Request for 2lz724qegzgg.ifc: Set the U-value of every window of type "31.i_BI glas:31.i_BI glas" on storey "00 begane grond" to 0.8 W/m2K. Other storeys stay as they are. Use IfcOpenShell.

First a look at what the model holds.

```python
import ifcopenshell
import ifcopenshell.util.element

model = ifcopenshell.open("2lz724qegzgg.ifc")
print(model.schema)
storey = next(s for s in model.by_type("IfcBuildingStorey") if s.Name == "00 begane grond")
windows = [e for e in ifcopenshell.util.element.get_decomposition(storey) if e.is_a("IfcWindow")]
seen = {}
for e in windows:
    element_type = ifcopenshell.util.element.get_type(e)
    key = (element_type.Name if element_type != e and element_type else None, ifcopenshell.util.element.get_pset(e, "Pset_WindowCommon", "ThermalTransmittance"))
    seen[key] = seen.get(key, 0) + 1
for (name, value), count in sorted(seen.items(), key=str):
    print(count, "x", name, "|", value)
```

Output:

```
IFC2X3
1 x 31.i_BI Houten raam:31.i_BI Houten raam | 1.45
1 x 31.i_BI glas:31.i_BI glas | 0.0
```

```python
import ifcopenshell
import ifcopenshell.api.pset
import ifcopenshell.util.element

model = ifcopenshell.open("2lz724qegzgg.ifc")

storey = next(s for s in model.by_type("IfcBuildingStorey") if s.Name == "00 begane grond")
windows = [e for e in ifcopenshell.util.element.get_decomposition(storey) if e.is_a("IfcWindow")]

count = 0
for e in windows:
    element_type = ifcopenshell.util.element.get_type(e)
    if element_type in (None, e) or element_type.Name != "31.i_BI glas:31.i_BI glas":
        continue
    # add_pset returns the element's existing set when there is one.
    pset = ifcopenshell.api.pset.add_pset(model, product=e, name="Pset_WindowCommon")
    ifcopenshell.api.pset.edit_pset(model, pset=pset, properties={"ThermalTransmittance": 0.8})
    count += 1

print(count, "windows updated")

model.write("2lz724qegzgg_edited.ifc")
```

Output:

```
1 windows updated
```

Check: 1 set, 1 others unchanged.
